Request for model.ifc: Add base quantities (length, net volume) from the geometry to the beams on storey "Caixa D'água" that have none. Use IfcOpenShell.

First a look at what the model holds.

```python
import ifcopenshell
import ifcopenshell.util.element
import ifcopenshell.util.unit

model = ifcopenshell.open("model.ifc")
print(model.schema)
for unit_type in ("LENGTHUNIT", "AREAUNIT", "VOLUMEUNIT"):
    print(unit_type, ifcopenshell.util.unit.calculate_unit_scale(model, unit_type))
storey = next(s for s in model.by_type("IfcBuildingStorey") if s.Name == "Caixa D'água")
beams = [e for e in ifcopenshell.util.element.get_decomposition(storey) if e.is_a("IfcBeam")]
for e in sorted(beams, key=lambda e: e.id()):
    print(e.id(), e.is_a(), e.Name, list(ifcopenshell.util.element.get_psets(e, qtos_only=True)), sep=" | ")
```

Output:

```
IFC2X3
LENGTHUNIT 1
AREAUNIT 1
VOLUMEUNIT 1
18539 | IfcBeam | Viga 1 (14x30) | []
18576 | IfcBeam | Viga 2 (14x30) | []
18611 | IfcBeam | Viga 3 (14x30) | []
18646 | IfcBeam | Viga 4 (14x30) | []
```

```python
import ifcopenshell
import ifcopenshell.api.pset
import ifcopenshell.geom
import ifcopenshell.util.element
import ifcopenshell.util.shape
import ifcopenshell.util.unit

model = ifcopenshell.open("model.ifc")
unit_scale = ifcopenshell.util.unit.calculate_unit_scale(model)
volume_scale = ifcopenshell.util.unit.calculate_unit_scale(model, "VOLUMEUNIT")
settings = ifcopenshell.geom.settings()

storey = next(s for s in model.by_type("IfcBuildingStorey") if s.Name == "Caixa D'água")
beams = [e for e in ifcopenshell.util.element.get_decomposition(storey) if e.is_a("IfcBeam")]

for e in sorted(beams, key=lambda e: e.id()):
    if ifcopenshell.util.element.get_psets(e, qtos_only=True, should_inherit=False):
        continue
    # Geometry comes back in metres, in the element's own axes.
    shape = ifcopenshell.geom.create_shape(settings, e)
    values = {
        "Length": ifcopenshell.util.shape.get_max_xyz(shape.geometry) / unit_scale,
        "NetVolume": ifcopenshell.util.shape.get_volume(shape.geometry) / volume_scale,
    }
    qto = ifcopenshell.api.pset.add_qto(model, product=e, name="BaseQuantities")
    ifcopenshell.api.pset.edit_qto(model, qto=qto, properties=values)
    print(e.id(), {k: round(v, 3) for k, v in values.items()})

model.write("model_rev.ifc")
```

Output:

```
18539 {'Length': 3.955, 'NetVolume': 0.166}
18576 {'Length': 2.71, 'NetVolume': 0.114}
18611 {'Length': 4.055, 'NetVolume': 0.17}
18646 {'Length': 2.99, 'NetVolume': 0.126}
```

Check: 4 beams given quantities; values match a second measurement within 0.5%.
